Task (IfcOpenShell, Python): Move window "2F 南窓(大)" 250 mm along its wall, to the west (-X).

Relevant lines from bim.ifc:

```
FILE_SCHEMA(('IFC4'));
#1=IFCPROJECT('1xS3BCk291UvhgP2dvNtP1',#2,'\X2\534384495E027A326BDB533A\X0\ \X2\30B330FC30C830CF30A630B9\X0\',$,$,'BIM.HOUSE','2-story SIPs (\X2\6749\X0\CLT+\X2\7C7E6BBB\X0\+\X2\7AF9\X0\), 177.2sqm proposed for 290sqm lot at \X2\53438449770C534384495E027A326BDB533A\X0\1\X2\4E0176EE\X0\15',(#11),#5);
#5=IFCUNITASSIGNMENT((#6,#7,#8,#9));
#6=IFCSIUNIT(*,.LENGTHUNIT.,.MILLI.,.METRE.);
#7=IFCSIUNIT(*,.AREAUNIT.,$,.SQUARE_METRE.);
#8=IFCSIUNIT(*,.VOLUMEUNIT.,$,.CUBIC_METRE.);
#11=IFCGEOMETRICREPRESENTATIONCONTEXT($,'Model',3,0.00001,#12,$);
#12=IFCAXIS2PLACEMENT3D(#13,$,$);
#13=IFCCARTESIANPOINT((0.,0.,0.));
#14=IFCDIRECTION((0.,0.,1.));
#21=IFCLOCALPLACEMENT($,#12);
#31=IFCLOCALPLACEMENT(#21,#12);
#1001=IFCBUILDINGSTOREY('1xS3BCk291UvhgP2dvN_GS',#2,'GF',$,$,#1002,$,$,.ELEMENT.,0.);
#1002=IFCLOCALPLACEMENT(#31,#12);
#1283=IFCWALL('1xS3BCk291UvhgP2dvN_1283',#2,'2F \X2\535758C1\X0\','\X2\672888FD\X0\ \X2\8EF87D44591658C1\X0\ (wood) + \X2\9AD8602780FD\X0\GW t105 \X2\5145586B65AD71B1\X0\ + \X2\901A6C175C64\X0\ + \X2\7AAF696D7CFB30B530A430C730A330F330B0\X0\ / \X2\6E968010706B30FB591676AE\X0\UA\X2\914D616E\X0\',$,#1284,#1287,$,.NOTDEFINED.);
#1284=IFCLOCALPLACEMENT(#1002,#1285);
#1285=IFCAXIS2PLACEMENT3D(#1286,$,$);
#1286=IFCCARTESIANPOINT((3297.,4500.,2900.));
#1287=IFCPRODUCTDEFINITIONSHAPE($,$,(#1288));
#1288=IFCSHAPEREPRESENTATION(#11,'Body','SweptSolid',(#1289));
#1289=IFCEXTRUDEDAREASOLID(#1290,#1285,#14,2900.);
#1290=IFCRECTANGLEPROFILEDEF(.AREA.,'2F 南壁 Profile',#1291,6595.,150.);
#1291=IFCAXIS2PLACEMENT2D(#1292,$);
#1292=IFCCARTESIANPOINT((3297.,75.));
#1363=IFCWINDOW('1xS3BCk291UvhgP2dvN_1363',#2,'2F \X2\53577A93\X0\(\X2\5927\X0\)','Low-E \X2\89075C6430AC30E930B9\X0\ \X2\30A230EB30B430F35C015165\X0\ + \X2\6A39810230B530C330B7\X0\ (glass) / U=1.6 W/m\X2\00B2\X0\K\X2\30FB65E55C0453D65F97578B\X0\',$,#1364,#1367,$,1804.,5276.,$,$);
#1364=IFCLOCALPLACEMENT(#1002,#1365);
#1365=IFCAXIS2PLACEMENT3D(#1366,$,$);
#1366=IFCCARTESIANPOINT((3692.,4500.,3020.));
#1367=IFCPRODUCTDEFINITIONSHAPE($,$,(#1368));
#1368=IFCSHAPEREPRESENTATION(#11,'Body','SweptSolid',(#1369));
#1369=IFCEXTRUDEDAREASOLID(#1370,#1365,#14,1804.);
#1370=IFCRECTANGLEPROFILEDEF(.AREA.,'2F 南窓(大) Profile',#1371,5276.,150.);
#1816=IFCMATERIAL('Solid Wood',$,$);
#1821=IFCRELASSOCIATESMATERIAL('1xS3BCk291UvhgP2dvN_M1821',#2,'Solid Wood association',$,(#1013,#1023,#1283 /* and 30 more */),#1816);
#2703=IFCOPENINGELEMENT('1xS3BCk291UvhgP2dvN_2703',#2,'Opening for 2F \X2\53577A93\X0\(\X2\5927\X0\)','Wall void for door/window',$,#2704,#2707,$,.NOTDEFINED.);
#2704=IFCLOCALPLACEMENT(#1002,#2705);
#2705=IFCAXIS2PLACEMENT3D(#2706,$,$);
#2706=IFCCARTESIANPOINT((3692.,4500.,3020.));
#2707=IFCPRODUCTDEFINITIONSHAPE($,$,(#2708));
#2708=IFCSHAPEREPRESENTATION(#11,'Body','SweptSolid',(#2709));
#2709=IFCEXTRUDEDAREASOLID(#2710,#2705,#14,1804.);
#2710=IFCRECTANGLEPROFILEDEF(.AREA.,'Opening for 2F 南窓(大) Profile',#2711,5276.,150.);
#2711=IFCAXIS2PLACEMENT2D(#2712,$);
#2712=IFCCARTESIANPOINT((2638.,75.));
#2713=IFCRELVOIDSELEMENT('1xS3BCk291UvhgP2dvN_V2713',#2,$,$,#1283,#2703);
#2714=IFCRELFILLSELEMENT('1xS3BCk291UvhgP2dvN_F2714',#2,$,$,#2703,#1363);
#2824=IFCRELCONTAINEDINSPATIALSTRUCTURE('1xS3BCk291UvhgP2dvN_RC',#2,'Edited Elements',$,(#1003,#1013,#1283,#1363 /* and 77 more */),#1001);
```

```python
import ifcopenshell
import ifcopenshell.api.geometry
import ifcopenshell.util.placement
import ifcopenshell.util.unit

model = ifcopenshell.open("bim.ifc")
unit_scale = ifcopenshell.util.unit.calculate_unit_scale(model)

window = model.by_guid("1xS3BCk291UvhgP2dvN_1363")
opening = window.FillsVoids[0].RelatingOpeningElement
wall = opening.VoidsElements[0].RelatingBuildingElement

wall_matrix = ifcopenshell.util.placement.get_local_placement(wall.ObjectPlacement)
shift = wall_matrix[:3, 0] * -0.25 / unit_scale
before = ifcopenshell.util.placement.get_local_placement(window.ObjectPlacement)[:3, 3].copy()

# The window is not placed relative to its opening, so move both.
for product in (opening, window):
    matrix = ifcopenshell.util.placement.get_local_placement(product.ObjectPlacement)
    matrix[:3, 3] += shift
    ifcopenshell.api.geometry.edit_object_placement(model, product=product, matrix=matrix, is_si=False)

after = ifcopenshell.util.placement.get_local_placement(window.ObjectPlacement)[:3, 3]
print("window moved by", (after - before).round(3) + 0.0)

model.write("bim-out.ifc")
```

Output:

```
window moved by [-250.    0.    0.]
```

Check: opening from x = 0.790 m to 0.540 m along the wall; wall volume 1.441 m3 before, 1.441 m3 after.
